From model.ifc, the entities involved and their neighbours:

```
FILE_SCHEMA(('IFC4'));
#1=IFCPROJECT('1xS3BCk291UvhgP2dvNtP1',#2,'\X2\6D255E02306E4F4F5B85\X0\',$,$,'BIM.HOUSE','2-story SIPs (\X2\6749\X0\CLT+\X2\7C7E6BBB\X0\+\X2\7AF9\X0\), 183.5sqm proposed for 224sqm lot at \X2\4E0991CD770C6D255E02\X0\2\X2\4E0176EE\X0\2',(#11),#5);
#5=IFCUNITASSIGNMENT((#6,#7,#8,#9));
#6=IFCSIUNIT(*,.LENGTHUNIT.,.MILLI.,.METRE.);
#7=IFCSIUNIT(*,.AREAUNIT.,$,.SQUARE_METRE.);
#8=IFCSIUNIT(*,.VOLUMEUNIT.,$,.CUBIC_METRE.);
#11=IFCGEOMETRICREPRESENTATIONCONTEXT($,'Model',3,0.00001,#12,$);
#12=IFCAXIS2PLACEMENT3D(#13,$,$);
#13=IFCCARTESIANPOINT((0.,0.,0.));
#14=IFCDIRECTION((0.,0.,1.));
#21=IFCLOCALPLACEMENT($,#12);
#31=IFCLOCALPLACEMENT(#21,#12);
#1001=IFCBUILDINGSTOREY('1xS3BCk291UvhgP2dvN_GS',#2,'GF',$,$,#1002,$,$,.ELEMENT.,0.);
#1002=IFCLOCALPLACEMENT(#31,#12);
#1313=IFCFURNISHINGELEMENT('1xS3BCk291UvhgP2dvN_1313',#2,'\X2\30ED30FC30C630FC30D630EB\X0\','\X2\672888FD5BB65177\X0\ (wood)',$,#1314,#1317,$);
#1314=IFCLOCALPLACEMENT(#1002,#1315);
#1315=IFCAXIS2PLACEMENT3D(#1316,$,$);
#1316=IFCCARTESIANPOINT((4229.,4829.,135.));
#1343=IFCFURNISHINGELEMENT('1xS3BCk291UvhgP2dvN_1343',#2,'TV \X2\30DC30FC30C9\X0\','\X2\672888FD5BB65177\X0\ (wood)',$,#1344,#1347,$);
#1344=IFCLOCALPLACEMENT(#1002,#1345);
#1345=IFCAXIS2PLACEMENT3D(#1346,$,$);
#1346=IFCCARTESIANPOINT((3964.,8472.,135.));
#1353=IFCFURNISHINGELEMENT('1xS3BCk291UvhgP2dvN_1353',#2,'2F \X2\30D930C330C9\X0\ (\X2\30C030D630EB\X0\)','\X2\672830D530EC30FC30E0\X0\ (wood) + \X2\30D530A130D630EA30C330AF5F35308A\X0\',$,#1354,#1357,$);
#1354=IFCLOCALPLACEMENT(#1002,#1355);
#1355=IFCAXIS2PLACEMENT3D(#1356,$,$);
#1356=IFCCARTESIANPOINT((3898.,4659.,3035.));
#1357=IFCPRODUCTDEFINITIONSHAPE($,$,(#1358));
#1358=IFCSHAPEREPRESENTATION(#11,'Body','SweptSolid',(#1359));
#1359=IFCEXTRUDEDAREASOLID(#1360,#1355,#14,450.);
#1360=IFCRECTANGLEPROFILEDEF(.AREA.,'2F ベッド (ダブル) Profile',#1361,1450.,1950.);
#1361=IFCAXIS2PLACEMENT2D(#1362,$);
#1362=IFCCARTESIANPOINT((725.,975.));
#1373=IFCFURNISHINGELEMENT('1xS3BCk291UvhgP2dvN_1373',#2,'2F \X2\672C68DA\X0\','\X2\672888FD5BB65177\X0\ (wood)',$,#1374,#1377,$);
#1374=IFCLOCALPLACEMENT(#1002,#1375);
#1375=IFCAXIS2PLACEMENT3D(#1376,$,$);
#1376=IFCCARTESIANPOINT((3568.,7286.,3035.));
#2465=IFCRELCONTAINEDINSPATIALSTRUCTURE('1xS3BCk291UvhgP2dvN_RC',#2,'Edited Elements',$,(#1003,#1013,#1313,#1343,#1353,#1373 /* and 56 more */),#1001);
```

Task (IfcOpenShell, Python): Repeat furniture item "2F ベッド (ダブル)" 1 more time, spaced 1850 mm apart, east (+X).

```python
import numpy as np
import ifcopenshell
import ifcopenshell.api.geometry
import ifcopenshell.api.root
import ifcopenshell.util.element
import ifcopenshell.util.placement
import ifcopenshell.util.unit

model = ifcopenshell.open("model.ifc")
unit_scale = ifcopenshell.util.unit.calculate_unit_scale(model)


def reuse_history(source, copy):
    """copy_class also copies each property set's owner history, people and application; keep the originals."""
    for rel in copy.IsDefinedBy:
        if rel.is_a("IfcRelDefinesByProperties") and (history := rel.RelatingPropertyDefinition.OwnerHistory):
            rel.RelatingPropertyDefinition.OwnerHistory = source.OwnerHistory
            ifcopenshell.util.element.remove_deep2(model, history)


source = model.by_guid("1xS3BCk291UvhgP2dvN_1353")
base = ifcopenshell.util.placement.get_local_placement(source.ObjectPlacement)
step = np.array([1.0, 0.0, 0.0]) * 1.85 / unit_scale

for i in range(1, 2):
    copy = ifcopenshell.api.root.copy_class(model, product=source)
    copy.Representation = ifcopenshell.util.element.copy_deep(
        model, source.Representation, exclude=["IfcGeometricRepresentationContext", "IfcRepresentationMap"]
    )
    reuse_history(source, copy)
    matrix = base.copy()
    matrix[:3, 3] += i * step
    print("added at", matrix[:3, 3].round(3) + 0.0)
    ifcopenshell.api.geometry.edit_object_placement(model, product=copy, matrix=matrix, is_si=False)

model.write("model_updated.ifc")
```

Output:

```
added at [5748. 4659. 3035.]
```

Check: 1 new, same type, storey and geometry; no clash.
